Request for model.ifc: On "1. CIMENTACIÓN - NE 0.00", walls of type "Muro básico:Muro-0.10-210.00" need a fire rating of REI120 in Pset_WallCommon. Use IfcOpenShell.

First a look at what the model holds.

```python
import ifcopenshell
import ifcopenshell.util.element

model = ifcopenshell.open("model.ifc")
print(model.schema)
storey = next(s for s in model.by_type("IfcBuildingStorey") if s.Name == "1. CIMENTACIÓN - NE 0.00")
walls = [e for e in ifcopenshell.util.element.get_decomposition(storey) if e.is_a("IfcWall")]
seen = {}
for e in walls:
    element_type = ifcopenshell.util.element.get_type(e)
    key = (element_type.Name if element_type != e and element_type else None, ifcopenshell.util.element.get_pset(e, "Pset_WallCommon", "FireRating"))
    seen[key] = seen.get(key, 0) + 1
for (name, value), count in sorted(seen.items(), key=str):
    print(count, "x", name, "|", value)
```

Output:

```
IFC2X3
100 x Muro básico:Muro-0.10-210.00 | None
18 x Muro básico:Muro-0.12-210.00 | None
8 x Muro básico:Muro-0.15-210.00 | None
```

```python
import ifcopenshell
import ifcopenshell.api.pset
import ifcopenshell.util.element

model = ifcopenshell.open("model.ifc")

storey = next(s for s in model.by_type("IfcBuildingStorey") if s.Name == "1. CIMENTACIÓN - NE 0.00")
walls = [e for e in ifcopenshell.util.element.get_decomposition(storey) if e.is_a("IfcWall")]

count = 0
for e in walls:
    element_type = ifcopenshell.util.element.get_type(e)
    if element_type in (None, e) or element_type.Name != "Muro básico:Muro-0.10-210.00":
        continue
    # add_pset returns the element's existing set when there is one.
    pset = ifcopenshell.api.pset.add_pset(model, product=e, name="Pset_WallCommon")
    ifcopenshell.api.pset.edit_pset(model, pset=pset, properties={"FireRating": "REI120"})
    count += 1

print(count, "walls updated")

model.write("model_edited.ifc")
```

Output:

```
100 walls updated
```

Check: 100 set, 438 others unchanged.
